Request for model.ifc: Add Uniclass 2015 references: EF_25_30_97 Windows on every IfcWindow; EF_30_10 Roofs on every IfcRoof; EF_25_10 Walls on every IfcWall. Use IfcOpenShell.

First a look at what the model holds.

```python
import ifcopenshell

model = ifcopenshell.open("model.ifc")
print(model.schema)
print("classifications:", [c.Name for c in model.by_type("IfcClassification")])
for ifc_class in ("IfcDoor", "IfcRoof", "IfcStair", "IfcWall", "IfcWindow"):
    print(ifc_class, len(model.by_type(ifc_class)))
```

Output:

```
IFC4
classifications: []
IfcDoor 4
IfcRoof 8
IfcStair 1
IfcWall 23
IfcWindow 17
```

```python
import ifcopenshell
import ifcopenshell.api.classification

model = ifcopenshell.open("model.ifc")

system = ifcopenshell.api.classification.add_classification(model, classification="Uniclass 2015")

codes = {
    "IfcWindow": ("EF_25_30_97", "Windows"),
    "IfcRoof": ("EF_30_10", "Roofs"),
    "IfcWall": ("EF_25_10", "Walls"),
}
for ifc_class, (code, name) in codes.items():
    products = model.by_type(ifc_class)
    ifcopenshell.api.classification.add_reference(
        model, products=products, classification=system, identification=code, name=name
    )
    print(code, len(products))

model.write("model_edited.ifc")
```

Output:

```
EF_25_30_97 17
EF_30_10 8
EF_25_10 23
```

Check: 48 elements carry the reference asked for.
